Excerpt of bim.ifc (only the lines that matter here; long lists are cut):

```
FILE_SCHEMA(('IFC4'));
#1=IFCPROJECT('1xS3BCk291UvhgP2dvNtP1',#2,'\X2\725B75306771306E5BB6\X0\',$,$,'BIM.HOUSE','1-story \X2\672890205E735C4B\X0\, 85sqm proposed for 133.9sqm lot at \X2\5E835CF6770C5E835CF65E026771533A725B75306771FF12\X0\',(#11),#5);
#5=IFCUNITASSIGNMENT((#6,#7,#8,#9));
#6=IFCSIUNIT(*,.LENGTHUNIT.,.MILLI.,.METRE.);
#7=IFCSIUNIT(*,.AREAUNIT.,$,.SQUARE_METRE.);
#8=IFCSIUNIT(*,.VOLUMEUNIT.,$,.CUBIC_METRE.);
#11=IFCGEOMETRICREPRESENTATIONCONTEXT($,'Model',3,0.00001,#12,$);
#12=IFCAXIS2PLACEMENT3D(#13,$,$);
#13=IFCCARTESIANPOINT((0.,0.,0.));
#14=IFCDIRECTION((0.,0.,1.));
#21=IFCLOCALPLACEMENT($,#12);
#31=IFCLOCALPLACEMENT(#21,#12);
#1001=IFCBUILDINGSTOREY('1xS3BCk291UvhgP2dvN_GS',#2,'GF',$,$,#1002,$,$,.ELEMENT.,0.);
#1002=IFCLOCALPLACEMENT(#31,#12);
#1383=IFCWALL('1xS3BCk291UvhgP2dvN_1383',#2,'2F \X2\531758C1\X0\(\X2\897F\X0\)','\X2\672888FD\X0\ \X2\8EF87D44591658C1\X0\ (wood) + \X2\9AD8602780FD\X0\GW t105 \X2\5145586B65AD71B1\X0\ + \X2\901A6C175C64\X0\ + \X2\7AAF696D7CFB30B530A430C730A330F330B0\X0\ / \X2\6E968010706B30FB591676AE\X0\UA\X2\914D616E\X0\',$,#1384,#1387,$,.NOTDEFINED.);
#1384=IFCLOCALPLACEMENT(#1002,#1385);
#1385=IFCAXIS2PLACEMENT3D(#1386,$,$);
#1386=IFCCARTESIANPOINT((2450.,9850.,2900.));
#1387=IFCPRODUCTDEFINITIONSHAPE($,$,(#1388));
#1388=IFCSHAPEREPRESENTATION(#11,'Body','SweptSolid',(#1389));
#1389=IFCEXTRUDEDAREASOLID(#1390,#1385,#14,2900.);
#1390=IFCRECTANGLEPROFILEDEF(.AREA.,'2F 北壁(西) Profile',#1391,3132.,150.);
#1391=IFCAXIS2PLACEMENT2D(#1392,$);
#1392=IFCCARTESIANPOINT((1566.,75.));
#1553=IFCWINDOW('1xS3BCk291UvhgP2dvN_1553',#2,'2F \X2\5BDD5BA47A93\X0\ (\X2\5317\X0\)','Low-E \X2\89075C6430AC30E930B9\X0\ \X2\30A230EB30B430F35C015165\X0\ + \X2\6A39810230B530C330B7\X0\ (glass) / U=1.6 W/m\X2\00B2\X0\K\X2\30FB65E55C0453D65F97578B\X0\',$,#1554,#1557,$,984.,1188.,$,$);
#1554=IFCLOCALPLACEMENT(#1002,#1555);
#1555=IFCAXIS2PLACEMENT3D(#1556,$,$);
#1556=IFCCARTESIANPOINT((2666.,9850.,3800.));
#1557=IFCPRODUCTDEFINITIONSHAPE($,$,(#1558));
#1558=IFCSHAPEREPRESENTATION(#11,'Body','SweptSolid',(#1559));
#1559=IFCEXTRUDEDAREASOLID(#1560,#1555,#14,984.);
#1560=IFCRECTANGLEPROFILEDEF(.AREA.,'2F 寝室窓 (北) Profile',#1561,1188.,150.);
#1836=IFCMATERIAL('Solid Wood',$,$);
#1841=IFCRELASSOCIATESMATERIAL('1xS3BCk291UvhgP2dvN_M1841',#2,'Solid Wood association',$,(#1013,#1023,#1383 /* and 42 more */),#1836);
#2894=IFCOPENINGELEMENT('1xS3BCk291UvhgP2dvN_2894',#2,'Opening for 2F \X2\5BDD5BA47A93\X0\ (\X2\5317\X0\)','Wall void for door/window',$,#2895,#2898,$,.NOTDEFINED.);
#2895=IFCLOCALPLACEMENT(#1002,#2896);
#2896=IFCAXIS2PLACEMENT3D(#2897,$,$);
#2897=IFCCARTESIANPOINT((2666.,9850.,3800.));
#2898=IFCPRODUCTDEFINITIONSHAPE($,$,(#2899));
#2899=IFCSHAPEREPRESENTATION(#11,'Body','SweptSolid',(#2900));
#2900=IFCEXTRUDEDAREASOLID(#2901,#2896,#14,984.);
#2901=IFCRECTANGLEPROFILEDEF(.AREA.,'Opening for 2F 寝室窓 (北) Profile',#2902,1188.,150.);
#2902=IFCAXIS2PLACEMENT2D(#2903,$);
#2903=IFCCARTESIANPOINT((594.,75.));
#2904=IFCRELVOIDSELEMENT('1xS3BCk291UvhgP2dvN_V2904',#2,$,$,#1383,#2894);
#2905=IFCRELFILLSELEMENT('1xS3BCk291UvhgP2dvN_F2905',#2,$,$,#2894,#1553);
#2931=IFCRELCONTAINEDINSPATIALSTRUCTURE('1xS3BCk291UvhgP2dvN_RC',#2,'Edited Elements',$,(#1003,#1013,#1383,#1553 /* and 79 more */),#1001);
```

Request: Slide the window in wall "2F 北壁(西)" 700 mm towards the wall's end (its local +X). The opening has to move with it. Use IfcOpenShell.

```python
import ifcopenshell
import ifcopenshell.api.geometry
import ifcopenshell.util.placement
import ifcopenshell.util.unit

model = ifcopenshell.open("bim.ifc")
unit_scale = ifcopenshell.util.unit.calculate_unit_scale(model)

window = model.by_id(1553)
opening = window.FillsVoids[0].RelatingOpeningElement
wall = opening.VoidsElements[0].RelatingBuildingElement

wall_matrix = ifcopenshell.util.placement.get_local_placement(wall.ObjectPlacement)
shift = wall_matrix[:3, 0] * 0.7 / unit_scale
before = ifcopenshell.util.placement.get_local_placement(window.ObjectPlacement)[:3, 3].copy()

# The window is not placed relative to its opening, so move both.
for product in (opening, window):
    matrix = ifcopenshell.util.placement.get_local_placement(product.ObjectPlacement)
    matrix[:3, 3] += shift
    ifcopenshell.api.geometry.edit_object_placement(model, product=product, matrix=matrix, is_si=False)

after = ifcopenshell.util.placement.get_local_placement(window.ObjectPlacement)[:3, 3]
print("window moved by", (after - before).round(3) + 0.0)

model.write("bim_edited.ifc")
```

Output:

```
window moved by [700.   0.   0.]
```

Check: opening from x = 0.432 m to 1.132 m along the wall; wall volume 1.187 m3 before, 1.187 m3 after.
